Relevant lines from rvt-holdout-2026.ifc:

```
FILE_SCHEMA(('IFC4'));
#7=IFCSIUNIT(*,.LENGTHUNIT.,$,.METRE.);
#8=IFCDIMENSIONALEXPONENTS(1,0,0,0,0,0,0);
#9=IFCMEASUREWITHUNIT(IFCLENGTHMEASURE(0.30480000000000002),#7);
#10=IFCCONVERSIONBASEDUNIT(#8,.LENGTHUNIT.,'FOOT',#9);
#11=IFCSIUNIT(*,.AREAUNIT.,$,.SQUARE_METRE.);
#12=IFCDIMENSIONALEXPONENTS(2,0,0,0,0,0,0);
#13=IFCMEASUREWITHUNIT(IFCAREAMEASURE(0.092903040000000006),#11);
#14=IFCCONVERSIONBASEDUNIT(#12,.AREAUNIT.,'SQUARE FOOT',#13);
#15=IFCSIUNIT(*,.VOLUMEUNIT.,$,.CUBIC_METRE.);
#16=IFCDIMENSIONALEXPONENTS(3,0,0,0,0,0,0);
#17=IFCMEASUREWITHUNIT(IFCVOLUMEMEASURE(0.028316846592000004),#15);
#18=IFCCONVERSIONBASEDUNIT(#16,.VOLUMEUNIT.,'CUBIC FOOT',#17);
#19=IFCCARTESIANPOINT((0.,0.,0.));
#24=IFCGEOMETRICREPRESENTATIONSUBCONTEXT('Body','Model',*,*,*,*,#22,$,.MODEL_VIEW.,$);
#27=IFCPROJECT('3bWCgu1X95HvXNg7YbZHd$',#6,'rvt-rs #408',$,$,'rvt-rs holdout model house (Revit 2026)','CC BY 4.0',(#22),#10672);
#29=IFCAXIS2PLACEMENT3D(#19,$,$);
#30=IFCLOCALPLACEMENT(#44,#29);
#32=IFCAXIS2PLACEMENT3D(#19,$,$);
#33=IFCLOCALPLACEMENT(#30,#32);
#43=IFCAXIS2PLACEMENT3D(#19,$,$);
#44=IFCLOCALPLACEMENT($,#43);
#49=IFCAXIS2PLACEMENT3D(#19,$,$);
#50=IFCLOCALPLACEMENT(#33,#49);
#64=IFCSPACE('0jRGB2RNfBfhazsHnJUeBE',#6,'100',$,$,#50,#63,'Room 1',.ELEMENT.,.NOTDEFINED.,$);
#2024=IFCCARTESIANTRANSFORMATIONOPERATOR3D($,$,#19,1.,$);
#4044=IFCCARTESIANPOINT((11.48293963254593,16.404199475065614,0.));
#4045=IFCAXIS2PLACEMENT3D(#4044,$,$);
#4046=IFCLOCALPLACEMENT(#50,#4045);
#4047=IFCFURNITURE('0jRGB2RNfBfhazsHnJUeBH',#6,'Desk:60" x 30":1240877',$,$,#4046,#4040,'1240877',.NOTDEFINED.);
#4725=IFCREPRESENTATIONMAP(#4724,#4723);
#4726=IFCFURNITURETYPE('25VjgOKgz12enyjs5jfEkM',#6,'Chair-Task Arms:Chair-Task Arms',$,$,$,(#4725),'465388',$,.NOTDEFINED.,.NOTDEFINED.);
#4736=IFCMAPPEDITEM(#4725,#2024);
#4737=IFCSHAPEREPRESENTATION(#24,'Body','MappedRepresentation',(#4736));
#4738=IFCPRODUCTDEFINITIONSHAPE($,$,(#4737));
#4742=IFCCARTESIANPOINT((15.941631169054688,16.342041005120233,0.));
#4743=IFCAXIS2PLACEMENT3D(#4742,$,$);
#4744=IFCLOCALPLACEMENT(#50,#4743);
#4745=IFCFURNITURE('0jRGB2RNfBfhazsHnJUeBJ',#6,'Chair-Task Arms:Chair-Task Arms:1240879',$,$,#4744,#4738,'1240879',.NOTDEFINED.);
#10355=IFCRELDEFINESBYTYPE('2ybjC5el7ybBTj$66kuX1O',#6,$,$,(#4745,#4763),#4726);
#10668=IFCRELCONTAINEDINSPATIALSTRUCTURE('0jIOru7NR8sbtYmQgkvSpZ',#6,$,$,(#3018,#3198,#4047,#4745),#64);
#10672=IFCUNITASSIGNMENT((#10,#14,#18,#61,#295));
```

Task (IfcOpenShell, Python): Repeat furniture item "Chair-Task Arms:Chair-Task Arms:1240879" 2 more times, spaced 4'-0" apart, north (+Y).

```python
import numpy as np
import ifcopenshell
import ifcopenshell.api.geometry
import ifcopenshell.api.root
import ifcopenshell.util.element
import ifcopenshell.util.placement
import ifcopenshell.util.unit

model = ifcopenshell.open("rvt-holdout-2026.ifc")
unit_scale = ifcopenshell.util.unit.calculate_unit_scale(model)


def reuse_history(source, copy):
    """copy_class also copies each property set's owner history, people and application; keep the originals."""
    for rel in copy.IsDefinedBy:
        if rel.is_a("IfcRelDefinesByProperties") and (history := rel.RelatingPropertyDefinition.OwnerHistory):
            rel.RelatingPropertyDefinition.OwnerHistory = source.OwnerHistory
            ifcopenshell.util.element.remove_deep2(model, history)


source = model.by_guid("0jRGB2RNfBfhazsHnJUeBJ")
base = ifcopenshell.util.placement.get_local_placement(source.ObjectPlacement)
step = np.array([0.0, 1.0, 0.0]) * 48 * 0.0254 / unit_scale

for i in range(1, 3):
    copy = ifcopenshell.api.root.copy_class(model, product=source)
    copy.Representation = ifcopenshell.util.element.copy_deep(
        model, source.Representation, exclude=["IfcGeometricRepresentationContext", "IfcRepresentationMap"]
    )
    copy.Name = "Chair-Task Arms:Chair-Task Arms"
    copy.Tag = None
    reuse_history(source, copy)
    matrix = base.copy()
    matrix[:3, 3] += i * step
    print("added at", matrix[:3, 3].round(3) + 0.0)
    ifcopenshell.api.geometry.edit_object_placement(model, product=copy, matrix=matrix, is_si=False)

model.write("rvt-holdout-2026-out.ifc")
```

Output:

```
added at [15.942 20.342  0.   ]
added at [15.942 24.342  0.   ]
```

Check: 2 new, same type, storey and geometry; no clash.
